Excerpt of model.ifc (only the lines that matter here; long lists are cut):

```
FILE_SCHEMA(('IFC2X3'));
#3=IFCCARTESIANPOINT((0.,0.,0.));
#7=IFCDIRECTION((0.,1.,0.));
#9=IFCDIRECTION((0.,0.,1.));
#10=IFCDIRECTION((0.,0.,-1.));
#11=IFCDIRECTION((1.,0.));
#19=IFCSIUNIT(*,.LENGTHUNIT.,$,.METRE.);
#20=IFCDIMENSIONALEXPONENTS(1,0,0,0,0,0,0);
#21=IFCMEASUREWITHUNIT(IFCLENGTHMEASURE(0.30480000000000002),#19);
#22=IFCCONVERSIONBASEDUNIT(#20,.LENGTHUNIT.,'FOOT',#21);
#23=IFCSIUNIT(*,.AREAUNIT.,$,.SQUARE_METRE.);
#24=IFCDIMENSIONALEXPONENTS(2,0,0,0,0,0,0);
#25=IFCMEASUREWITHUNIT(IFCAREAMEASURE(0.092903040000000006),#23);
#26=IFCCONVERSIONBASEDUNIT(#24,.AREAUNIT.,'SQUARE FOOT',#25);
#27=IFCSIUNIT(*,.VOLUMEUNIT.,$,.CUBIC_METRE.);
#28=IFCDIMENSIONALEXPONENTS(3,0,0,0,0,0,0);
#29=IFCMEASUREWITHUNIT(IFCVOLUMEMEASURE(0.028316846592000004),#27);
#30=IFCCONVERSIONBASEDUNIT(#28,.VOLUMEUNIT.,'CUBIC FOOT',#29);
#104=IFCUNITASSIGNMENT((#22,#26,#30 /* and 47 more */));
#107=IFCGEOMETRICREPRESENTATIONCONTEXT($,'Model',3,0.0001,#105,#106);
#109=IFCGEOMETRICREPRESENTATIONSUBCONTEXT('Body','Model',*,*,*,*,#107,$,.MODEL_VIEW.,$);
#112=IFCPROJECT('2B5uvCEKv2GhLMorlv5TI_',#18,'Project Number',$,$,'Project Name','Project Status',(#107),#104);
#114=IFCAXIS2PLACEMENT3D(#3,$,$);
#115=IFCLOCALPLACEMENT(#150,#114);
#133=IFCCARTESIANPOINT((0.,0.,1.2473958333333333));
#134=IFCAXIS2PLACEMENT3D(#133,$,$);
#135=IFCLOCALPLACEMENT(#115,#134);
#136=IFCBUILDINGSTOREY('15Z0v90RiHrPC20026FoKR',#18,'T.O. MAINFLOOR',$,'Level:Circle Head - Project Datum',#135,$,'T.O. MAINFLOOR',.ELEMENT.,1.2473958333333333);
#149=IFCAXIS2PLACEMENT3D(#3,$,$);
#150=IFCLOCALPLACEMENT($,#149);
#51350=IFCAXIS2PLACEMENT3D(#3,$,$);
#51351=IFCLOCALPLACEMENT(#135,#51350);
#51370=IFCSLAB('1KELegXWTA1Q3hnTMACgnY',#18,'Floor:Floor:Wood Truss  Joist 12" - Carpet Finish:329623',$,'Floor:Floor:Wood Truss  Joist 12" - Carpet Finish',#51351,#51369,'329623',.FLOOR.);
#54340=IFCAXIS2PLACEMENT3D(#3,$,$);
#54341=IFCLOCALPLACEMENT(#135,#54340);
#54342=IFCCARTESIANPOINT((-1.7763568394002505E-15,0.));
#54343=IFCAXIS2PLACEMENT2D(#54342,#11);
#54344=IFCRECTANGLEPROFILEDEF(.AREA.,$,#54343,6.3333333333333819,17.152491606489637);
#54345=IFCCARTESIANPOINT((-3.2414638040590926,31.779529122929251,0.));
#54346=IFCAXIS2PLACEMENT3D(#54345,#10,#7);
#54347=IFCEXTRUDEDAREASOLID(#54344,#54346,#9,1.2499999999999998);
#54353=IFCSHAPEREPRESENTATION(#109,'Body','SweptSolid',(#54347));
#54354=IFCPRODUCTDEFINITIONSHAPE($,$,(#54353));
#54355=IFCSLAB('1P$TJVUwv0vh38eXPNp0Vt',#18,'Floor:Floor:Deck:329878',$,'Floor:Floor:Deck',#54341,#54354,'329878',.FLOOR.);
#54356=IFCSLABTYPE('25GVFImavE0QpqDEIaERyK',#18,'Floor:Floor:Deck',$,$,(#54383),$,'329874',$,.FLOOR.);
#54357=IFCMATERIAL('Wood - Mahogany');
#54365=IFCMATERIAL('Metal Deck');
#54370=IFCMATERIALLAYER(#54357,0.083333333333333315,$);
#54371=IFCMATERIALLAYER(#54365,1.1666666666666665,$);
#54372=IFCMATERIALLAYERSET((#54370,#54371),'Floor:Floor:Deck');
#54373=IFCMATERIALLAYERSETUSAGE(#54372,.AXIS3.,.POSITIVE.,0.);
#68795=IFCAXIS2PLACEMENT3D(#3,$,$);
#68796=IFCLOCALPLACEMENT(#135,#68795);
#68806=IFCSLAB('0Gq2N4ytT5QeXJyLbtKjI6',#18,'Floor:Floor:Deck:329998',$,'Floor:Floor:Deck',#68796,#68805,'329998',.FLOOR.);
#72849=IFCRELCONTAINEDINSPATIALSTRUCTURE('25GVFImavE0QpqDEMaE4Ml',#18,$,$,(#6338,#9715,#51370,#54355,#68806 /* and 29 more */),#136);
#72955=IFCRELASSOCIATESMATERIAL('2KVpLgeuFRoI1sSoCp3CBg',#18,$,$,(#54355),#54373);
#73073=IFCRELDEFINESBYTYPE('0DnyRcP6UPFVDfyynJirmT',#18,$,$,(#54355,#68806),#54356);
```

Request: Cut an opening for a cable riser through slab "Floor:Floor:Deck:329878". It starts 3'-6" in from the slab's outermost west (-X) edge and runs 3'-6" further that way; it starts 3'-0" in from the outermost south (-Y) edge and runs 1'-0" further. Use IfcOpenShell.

```python
import numpy as np
import ifcopenshell
import ifcopenshell.api.feature
import ifcopenshell.api.geometry
import ifcopenshell.api.root
import ifcopenshell.geom
import ifcopenshell.util.placement
import ifcopenshell.util.representation
import ifcopenshell.util.shape
import ifcopenshell.util.unit

model = ifcopenshell.open("model.ifc")
unit_scale = ifcopenshell.util.unit.calculate_unit_scale(model)
settings = ifcopenshell.geom.settings()


def volume(element):
    """Net volume in cubic metres, openings subtracted."""
    shape = ifcopenshell.geom.create_shape(settings, element)
    return ifcopenshell.util.shape.get_volume(shape.geometry)


slab = model.by_guid("1P$TJVUwv0vh38eXPNp0Vt")
before = volume(slab)

# Extent in the slab's own axes, in metres. The edges named are its -X and -Y sides.
slab_shape = ifcopenshell.geom.create_shape(settings, slab)
vertices = ifcopenshell.util.shape.get_vertices(slab_shape.geometry)
x_min, y_min, bottom = vertices.min(axis=0)
top = vertices[:, 2].max()

opening = ifcopenshell.api.root.create_entity(model, ifc_class="IfcOpeningElement", name="Cable riser opening")
context = ifcopenshell.util.representation.get_context(model, "Model", "Body", "MODEL_VIEW")
width, depth = 1.0668, 0.3048
outline = [(0.0, 0.0), (width, 0.0), (width, depth), (0.0, depth), (0.0, 0.0)]
# Overshoot both faces by 50 mm so the cut is clean.
shape = ifcopenshell.api.geometry.add_slab_representation(
    model, context=context, depth=top - bottom + 0.1, polyline=outline
)
ifcopenshell.api.geometry.assign_representation(model, product=opening, representation=shape)

matrix = ifcopenshell.util.placement.get_local_placement(slab.ObjectPlacement)
matrix[:, 3] = matrix @ np.append(np.array([x_min + 1.0668, y_min + 0.9144, bottom - 0.05]) / unit_scale, 1.0)
ifcopenshell.api.geometry.edit_object_placement(model, product=opening, matrix=matrix, is_si=False)
ifcopenshell.api.feature.add_feature(model, feature=opening, element=slab)

after = volume(slab)

print(f"slab volume {before:.3f} -> {after:.3f} m3")

model.write("model_v2.ifc")
```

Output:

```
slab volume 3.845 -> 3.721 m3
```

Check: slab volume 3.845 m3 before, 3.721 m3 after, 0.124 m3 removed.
